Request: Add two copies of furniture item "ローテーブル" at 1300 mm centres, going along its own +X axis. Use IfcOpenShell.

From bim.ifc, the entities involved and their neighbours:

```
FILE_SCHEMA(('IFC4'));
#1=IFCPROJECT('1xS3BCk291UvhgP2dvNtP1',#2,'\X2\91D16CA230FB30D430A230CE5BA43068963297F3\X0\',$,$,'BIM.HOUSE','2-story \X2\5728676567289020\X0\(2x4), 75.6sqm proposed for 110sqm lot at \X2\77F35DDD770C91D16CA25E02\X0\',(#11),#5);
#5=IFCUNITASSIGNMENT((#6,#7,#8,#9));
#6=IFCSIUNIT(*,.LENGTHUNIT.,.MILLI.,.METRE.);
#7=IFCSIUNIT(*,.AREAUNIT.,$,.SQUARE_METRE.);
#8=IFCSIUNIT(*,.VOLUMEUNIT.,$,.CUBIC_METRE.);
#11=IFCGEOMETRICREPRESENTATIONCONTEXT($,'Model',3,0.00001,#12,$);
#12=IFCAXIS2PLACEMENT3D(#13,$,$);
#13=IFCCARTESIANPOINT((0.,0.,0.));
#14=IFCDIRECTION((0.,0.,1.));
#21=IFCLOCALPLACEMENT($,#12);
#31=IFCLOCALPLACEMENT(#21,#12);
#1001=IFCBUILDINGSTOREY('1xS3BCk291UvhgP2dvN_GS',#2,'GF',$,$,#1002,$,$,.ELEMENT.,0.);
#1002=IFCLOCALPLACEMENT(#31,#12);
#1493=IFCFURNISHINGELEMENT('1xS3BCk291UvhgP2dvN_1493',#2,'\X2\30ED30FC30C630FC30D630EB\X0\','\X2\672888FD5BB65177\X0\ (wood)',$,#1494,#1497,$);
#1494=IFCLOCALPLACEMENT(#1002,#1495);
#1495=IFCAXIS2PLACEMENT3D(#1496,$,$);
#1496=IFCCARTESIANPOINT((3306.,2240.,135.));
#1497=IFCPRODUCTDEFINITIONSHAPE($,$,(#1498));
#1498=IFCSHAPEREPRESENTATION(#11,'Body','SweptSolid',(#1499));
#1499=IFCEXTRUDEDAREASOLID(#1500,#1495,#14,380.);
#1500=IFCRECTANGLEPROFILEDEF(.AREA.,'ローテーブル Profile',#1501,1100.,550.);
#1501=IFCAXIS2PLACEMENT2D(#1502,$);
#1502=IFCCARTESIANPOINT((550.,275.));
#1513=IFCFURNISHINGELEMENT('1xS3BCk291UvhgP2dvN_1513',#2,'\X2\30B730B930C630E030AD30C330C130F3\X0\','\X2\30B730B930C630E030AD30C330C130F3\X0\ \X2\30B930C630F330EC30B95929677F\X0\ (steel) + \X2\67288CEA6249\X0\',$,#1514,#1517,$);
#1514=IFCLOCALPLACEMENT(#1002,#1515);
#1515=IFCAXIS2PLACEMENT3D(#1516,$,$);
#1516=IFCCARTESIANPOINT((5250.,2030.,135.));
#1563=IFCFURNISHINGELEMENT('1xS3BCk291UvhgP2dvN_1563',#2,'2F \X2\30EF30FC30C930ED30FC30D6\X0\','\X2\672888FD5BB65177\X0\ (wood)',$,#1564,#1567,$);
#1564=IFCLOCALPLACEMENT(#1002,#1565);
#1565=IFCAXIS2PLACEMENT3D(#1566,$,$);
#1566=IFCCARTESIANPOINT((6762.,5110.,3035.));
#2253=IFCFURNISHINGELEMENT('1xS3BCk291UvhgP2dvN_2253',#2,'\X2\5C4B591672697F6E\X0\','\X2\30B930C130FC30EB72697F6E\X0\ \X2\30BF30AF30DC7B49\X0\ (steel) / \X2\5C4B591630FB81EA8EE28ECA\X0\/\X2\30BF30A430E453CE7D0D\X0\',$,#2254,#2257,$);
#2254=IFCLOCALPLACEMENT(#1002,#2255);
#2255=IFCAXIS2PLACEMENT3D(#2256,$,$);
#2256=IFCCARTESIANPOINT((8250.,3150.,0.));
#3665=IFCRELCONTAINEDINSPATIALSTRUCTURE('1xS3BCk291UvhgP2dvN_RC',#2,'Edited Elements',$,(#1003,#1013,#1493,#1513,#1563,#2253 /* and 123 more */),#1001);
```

```python
import ifcopenshell
import ifcopenshell.api.geometry
import ifcopenshell.api.root
import ifcopenshell.util.element
import ifcopenshell.util.placement

model = ifcopenshell.open("bim.ifc")


def reuse_history(source, copy):
    """copy_class also copies each property set's owner history, people and application; keep the originals."""
    for rel in copy.IsDefinedBy:
        if rel.is_a("IfcRelDefinesByProperties") and (history := rel.RelatingPropertyDefinition.OwnerHistory):
            rel.RelatingPropertyDefinition.OwnerHistory = source.OwnerHistory
            ifcopenshell.util.element.remove_deep2(model, history)


source = model.by_guid("1xS3BCk291UvhgP2dvN_1493")
base = ifcopenshell.util.placement.get_local_placement(source.ObjectPlacement)
step = base[:3, 0] * 1300.0

for i in range(1, 3):
    copy = ifcopenshell.api.root.copy_class(model, product=source)
    copy.Representation = ifcopenshell.util.element.copy_deep(
        model, source.Representation, exclude=["IfcGeometricRepresentationContext", "IfcRepresentationMap"]
    )
    reuse_history(source, copy)
    matrix = base.copy()
    matrix[:3, 3] += i * step
    print("added at", matrix[:3, 3].round(3) + 0.0)
    ifcopenshell.api.geometry.edit_object_placement(model, product=copy, matrix=matrix, is_si=False)

model.write("bim_rev.ifc")
```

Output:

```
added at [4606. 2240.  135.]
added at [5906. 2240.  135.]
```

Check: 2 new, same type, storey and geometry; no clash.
